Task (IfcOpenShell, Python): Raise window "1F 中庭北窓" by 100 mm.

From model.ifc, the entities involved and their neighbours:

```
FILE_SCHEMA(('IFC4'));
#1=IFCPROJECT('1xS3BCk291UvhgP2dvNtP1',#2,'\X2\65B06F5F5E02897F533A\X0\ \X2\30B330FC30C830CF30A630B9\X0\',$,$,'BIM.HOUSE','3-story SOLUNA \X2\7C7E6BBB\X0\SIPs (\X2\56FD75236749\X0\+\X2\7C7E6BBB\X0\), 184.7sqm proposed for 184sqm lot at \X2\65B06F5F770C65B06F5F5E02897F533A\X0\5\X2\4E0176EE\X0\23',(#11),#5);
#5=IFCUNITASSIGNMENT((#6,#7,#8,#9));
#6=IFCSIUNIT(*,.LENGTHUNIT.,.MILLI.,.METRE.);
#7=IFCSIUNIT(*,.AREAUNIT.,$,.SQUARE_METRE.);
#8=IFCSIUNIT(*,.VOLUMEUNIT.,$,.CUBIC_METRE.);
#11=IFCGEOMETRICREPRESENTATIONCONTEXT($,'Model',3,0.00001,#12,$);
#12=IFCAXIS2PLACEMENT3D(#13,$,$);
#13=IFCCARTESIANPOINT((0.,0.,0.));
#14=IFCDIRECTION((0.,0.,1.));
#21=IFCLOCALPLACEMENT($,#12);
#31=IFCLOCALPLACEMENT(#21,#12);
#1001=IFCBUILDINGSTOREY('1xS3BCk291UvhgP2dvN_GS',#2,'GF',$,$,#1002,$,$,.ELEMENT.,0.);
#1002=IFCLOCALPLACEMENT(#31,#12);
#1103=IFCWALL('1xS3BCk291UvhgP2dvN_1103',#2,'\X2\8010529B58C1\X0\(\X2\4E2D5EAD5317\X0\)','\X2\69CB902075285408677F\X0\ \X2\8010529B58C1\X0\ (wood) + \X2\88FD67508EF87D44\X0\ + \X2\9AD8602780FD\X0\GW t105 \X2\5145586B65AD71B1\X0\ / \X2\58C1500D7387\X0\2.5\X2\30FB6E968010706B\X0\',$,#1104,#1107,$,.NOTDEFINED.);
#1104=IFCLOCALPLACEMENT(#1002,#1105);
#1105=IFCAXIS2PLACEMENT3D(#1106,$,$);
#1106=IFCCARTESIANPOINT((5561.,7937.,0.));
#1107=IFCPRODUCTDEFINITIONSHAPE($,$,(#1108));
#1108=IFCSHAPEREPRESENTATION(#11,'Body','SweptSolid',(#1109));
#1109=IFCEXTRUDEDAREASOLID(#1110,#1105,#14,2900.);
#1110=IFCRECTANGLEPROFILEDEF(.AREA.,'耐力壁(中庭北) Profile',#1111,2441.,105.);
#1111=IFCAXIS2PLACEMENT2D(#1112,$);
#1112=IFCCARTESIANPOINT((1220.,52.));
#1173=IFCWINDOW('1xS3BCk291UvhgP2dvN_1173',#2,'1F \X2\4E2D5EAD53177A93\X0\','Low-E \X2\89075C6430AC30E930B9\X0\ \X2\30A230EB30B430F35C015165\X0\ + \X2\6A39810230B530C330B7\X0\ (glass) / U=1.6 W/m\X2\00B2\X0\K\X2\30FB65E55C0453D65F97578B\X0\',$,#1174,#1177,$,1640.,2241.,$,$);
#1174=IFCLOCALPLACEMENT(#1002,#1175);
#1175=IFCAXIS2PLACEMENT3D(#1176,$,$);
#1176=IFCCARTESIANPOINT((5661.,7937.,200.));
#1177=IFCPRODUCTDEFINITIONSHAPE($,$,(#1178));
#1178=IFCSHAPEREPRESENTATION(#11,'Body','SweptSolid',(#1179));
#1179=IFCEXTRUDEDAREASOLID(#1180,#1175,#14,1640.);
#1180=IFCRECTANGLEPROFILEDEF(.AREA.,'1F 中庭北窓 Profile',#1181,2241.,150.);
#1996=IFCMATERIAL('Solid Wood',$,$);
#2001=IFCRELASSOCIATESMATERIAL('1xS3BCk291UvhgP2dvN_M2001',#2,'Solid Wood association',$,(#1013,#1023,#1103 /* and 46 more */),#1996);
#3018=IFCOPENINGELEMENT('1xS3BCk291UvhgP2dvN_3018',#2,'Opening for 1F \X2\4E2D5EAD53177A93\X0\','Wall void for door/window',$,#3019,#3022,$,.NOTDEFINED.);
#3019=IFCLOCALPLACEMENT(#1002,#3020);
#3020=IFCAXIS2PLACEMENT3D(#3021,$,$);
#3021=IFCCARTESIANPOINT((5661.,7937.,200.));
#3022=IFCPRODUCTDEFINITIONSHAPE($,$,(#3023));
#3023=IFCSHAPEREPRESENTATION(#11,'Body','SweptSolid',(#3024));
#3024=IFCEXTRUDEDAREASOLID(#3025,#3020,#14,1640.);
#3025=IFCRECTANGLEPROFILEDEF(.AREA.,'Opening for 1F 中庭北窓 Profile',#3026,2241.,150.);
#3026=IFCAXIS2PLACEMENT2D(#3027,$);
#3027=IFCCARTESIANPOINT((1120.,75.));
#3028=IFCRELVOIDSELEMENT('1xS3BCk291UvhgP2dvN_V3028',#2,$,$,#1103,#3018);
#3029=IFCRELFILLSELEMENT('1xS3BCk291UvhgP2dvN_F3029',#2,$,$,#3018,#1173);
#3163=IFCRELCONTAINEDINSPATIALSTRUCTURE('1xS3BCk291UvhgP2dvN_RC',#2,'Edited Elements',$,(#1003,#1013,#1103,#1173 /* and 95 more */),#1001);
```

```python
import numpy as np
import ifcopenshell
import ifcopenshell.api.geometry
import ifcopenshell.util.placement
import ifcopenshell.util.unit

model = ifcopenshell.open("model.ifc")
unit_scale = ifcopenshell.util.unit.calculate_unit_scale(model)

window = model.by_guid("1xS3BCk291UvhgP2dvN_1173")
opening = window.FillsVoids[0].RelatingOpeningElement
dz = 0.1 / unit_scale

shift = np.array([0.0, 0.0, dz])
# The window is not placed relative to its opening, so move both.
for product in (opening, window):
    matrix = ifcopenshell.util.placement.get_local_placement(product.ObjectPlacement)
    matrix[:3, 3] += shift
    ifcopenshell.api.geometry.edit_object_placement(model, product=product, matrix=matrix, is_si=False)

print(f"moved by {dz * unit_scale:+.3f} m")

model.write("model-out.ifc")
```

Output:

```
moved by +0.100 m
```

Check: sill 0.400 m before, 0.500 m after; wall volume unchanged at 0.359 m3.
